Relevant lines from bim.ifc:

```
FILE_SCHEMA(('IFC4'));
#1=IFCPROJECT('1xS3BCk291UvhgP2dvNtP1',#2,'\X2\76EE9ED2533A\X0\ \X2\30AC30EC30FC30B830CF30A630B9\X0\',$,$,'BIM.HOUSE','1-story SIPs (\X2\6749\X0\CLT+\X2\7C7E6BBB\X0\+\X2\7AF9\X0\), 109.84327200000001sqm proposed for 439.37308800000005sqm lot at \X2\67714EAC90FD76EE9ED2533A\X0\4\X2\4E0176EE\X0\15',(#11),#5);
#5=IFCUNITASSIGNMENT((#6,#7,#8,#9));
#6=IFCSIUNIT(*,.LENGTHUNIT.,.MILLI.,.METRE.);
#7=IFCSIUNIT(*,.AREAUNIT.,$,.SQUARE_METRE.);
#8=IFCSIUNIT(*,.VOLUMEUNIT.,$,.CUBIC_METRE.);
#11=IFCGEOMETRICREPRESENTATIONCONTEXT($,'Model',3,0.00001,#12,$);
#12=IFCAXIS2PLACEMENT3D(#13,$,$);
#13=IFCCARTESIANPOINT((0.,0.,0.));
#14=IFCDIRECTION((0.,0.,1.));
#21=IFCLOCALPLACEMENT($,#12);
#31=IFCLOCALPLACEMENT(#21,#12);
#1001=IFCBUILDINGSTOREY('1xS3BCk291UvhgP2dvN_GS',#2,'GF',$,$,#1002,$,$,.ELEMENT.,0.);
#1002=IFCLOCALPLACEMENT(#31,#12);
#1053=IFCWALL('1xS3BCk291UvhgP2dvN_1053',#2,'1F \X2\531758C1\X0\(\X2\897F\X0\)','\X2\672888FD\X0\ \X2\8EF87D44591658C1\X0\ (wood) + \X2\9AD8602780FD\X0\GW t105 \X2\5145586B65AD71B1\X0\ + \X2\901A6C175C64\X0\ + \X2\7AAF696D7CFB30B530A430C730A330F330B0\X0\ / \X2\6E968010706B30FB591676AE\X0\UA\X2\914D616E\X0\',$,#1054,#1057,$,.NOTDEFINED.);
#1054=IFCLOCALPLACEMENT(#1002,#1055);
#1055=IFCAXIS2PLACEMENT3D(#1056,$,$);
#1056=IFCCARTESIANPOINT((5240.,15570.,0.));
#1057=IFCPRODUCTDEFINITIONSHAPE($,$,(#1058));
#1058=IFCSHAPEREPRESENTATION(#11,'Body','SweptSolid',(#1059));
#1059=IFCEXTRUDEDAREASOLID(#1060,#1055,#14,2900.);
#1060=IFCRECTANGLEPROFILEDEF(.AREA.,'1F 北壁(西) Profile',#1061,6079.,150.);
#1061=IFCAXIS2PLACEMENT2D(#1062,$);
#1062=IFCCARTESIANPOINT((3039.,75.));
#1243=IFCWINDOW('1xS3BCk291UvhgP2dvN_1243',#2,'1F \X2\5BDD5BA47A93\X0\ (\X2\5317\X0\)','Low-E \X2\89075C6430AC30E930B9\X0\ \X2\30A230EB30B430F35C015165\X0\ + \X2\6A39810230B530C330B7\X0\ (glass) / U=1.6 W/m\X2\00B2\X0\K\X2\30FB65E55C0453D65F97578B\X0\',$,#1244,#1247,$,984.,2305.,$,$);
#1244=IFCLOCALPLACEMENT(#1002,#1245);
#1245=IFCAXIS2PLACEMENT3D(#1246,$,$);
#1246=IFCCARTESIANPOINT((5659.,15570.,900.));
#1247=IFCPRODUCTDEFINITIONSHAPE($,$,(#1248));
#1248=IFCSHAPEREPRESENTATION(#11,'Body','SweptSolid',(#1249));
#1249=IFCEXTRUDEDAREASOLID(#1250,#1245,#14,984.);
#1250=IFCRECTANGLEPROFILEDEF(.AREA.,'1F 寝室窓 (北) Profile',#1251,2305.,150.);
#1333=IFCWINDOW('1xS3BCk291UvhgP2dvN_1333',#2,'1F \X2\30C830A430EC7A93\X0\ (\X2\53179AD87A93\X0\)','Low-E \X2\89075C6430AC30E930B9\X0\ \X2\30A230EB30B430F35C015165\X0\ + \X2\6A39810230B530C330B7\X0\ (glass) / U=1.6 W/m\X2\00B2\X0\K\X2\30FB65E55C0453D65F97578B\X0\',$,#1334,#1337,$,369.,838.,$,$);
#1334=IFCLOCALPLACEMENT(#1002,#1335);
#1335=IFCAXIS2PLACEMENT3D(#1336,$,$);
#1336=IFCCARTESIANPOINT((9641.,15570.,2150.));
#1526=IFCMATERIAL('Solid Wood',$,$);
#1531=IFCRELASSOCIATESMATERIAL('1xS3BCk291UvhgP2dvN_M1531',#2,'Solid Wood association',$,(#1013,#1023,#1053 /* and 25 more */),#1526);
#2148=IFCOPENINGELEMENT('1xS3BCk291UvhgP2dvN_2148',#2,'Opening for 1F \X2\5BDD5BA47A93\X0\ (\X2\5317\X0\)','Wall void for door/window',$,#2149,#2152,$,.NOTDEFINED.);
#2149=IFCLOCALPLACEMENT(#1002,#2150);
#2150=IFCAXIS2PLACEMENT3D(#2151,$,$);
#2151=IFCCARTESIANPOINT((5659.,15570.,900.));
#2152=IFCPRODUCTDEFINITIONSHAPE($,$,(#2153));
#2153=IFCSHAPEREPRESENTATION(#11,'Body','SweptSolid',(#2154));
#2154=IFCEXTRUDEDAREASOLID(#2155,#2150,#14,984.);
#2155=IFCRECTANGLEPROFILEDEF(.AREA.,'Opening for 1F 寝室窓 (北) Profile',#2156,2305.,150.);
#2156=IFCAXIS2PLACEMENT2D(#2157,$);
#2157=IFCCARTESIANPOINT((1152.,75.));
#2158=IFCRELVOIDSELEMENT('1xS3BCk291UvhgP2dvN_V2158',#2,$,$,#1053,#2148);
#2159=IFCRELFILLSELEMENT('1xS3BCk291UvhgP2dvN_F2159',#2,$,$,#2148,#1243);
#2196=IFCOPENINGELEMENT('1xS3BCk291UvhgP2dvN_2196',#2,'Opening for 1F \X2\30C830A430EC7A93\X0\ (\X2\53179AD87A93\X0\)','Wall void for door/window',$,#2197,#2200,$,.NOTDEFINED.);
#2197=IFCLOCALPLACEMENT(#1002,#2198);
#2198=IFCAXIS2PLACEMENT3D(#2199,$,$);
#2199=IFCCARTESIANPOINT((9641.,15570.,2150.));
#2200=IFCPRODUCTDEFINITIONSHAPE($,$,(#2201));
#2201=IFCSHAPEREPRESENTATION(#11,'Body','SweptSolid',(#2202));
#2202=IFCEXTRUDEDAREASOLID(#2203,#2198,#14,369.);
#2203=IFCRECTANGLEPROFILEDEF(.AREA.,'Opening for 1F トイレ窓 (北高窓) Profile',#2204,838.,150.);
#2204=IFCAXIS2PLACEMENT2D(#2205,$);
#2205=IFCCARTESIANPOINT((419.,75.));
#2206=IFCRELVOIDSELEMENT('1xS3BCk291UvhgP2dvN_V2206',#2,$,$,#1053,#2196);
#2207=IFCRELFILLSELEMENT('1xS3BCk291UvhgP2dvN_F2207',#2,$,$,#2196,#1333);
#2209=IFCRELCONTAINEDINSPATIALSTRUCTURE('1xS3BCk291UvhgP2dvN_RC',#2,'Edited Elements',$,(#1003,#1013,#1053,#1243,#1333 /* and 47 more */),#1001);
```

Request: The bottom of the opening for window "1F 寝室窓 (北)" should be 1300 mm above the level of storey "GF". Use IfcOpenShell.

```python
import numpy as np
import ifcopenshell
import ifcopenshell.api.geometry
import ifcopenshell.geom
import ifcopenshell.util.element
import ifcopenshell.util.placement
import ifcopenshell.util.shape
import ifcopenshell.util.unit

model = ifcopenshell.open("bim.ifc")
unit_scale = ifcopenshell.util.unit.calculate_unit_scale(model)

window = model.by_guid("1xS3BCk291UvhgP2dvN_1243")
opening = window.FillsVoids[0].RelatingOpeningElement
storey = ifcopenshell.util.element.get_container(window, ifc_class="IfcBuildingStorey")
level = ifcopenshell.util.placement.get_local_placement(storey.ObjectPlacement)[2, 3]

# The opening's origin need not be at the sill, so measure its lowest point.
shape = ifcopenshell.geom.create_shape(ifcopenshell.geom.settings(), opening)
bottom = ifcopenshell.util.shape.get_shape_bottom_elevation(shape, shape.geometry) / unit_scale
dz = level + 1.3 / unit_scale - bottom

shift = np.array([0.0, 0.0, dz])
# The window is not placed relative to its opening, so move both.
for product in (opening, window):
    matrix = ifcopenshell.util.placement.get_local_placement(product.ObjectPlacement)
    matrix[:3, 3] += shift
    ifcopenshell.api.geometry.edit_object_placement(model, product=product, matrix=matrix, is_si=False)

print(f"moved by {dz * unit_scale:+.3f} m")

model.write("bim-out.ifc")
```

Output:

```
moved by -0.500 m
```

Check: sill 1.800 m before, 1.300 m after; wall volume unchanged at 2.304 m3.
